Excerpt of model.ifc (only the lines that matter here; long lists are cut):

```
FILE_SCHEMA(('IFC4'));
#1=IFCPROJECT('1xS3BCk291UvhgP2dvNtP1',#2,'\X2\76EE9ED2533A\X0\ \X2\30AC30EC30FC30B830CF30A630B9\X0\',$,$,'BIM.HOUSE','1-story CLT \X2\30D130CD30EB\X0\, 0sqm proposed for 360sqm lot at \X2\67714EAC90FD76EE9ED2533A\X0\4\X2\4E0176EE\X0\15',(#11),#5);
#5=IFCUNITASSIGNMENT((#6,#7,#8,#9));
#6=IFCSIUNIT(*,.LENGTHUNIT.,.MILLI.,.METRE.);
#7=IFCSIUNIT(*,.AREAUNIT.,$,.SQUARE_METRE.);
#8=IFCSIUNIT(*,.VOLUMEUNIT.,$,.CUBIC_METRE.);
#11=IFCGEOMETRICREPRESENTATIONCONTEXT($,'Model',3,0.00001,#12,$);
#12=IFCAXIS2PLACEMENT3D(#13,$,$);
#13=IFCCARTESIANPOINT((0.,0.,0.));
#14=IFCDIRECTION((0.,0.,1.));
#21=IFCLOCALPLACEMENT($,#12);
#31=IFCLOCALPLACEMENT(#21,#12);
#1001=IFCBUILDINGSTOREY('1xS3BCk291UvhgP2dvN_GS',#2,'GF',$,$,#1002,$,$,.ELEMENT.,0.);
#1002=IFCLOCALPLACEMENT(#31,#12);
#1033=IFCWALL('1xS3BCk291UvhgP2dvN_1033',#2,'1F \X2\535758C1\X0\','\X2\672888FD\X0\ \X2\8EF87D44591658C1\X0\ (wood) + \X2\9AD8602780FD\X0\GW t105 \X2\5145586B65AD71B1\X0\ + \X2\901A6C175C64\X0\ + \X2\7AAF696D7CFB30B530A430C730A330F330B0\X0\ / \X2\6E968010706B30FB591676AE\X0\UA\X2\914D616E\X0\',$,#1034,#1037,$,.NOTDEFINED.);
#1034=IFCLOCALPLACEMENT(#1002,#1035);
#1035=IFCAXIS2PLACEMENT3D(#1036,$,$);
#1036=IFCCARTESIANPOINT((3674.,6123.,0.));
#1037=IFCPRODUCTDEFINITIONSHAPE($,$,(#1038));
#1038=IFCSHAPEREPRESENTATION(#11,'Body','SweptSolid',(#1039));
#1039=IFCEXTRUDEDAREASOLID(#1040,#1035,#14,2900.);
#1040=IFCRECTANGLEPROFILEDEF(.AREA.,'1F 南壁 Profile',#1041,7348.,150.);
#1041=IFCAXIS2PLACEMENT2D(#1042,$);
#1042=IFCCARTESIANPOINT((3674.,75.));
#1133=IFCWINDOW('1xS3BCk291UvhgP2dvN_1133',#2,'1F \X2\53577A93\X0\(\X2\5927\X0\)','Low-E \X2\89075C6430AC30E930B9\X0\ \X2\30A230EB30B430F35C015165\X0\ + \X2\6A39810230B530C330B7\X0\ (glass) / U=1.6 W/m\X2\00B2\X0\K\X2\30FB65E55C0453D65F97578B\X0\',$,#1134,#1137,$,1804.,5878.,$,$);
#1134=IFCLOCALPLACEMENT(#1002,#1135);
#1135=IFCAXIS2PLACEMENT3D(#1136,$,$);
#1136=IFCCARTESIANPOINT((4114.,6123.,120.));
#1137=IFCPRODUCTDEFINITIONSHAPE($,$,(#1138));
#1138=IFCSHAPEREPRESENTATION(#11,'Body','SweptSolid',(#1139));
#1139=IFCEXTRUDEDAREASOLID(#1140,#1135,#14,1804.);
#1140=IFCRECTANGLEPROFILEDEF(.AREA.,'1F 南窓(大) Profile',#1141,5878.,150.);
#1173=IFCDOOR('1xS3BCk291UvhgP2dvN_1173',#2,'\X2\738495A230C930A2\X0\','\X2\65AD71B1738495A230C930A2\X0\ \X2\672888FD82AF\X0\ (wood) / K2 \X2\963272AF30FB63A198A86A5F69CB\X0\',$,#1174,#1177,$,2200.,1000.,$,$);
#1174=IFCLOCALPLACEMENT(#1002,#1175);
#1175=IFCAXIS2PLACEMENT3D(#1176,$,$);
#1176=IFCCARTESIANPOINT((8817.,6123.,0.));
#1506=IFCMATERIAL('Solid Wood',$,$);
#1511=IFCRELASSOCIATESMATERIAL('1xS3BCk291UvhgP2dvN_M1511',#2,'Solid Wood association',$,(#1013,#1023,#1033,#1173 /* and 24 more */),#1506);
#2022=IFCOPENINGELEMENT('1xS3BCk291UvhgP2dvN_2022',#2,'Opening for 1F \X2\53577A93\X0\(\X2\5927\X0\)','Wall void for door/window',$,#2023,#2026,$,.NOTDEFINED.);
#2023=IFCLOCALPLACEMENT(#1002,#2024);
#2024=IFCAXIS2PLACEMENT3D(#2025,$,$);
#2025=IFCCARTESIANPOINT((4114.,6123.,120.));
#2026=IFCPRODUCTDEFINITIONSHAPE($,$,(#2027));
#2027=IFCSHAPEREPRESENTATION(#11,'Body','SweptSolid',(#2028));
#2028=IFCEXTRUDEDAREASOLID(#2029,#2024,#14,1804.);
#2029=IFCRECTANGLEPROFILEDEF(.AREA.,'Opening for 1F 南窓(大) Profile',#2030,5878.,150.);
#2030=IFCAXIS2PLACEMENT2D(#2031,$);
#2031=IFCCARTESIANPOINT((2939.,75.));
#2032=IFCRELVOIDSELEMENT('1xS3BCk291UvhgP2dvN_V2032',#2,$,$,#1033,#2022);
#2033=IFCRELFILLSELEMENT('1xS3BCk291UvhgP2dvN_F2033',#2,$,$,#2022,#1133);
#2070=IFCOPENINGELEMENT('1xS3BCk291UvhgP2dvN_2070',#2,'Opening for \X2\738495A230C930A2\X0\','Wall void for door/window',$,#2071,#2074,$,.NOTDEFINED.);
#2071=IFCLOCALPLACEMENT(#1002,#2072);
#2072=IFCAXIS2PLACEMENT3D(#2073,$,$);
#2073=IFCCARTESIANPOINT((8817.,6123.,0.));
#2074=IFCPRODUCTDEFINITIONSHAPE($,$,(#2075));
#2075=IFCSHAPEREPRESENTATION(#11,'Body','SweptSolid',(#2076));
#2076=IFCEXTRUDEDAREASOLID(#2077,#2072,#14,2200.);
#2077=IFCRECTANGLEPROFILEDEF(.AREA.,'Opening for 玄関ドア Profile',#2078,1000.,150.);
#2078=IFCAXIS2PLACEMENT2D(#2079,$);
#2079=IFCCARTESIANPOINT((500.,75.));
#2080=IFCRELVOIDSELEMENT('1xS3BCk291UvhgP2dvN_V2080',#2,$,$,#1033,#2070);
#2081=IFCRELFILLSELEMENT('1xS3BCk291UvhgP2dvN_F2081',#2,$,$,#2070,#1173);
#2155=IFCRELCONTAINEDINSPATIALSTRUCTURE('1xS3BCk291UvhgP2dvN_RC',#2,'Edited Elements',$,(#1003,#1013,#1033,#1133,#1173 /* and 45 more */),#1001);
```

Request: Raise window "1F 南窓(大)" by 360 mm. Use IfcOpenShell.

```python
import numpy as np
import ifcopenshell
import ifcopenshell.api.geometry
import ifcopenshell.util.placement
import ifcopenshell.util.unit

model = ifcopenshell.open("model.ifc")
unit_scale = ifcopenshell.util.unit.calculate_unit_scale(model)

window = model.by_guid("1xS3BCk291UvhgP2dvN_1133")
opening = window.FillsVoids[0].RelatingOpeningElement
dz = 0.36 / unit_scale

shift = np.array([0.0, 0.0, dz])
# The window is not placed relative to its opening, so move both.
for product in (opening, window):
    matrix = ifcopenshell.util.placement.get_local_placement(product.ObjectPlacement)
    matrix[:3, 3] += shift
    ifcopenshell.api.geometry.edit_object_placement(model, product=product, matrix=matrix, is_si=False)

print(f"moved by {dz * unit_scale:+.3f} m")

model.write("model_v2.ifc")
```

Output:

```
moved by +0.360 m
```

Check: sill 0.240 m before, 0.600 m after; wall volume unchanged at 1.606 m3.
